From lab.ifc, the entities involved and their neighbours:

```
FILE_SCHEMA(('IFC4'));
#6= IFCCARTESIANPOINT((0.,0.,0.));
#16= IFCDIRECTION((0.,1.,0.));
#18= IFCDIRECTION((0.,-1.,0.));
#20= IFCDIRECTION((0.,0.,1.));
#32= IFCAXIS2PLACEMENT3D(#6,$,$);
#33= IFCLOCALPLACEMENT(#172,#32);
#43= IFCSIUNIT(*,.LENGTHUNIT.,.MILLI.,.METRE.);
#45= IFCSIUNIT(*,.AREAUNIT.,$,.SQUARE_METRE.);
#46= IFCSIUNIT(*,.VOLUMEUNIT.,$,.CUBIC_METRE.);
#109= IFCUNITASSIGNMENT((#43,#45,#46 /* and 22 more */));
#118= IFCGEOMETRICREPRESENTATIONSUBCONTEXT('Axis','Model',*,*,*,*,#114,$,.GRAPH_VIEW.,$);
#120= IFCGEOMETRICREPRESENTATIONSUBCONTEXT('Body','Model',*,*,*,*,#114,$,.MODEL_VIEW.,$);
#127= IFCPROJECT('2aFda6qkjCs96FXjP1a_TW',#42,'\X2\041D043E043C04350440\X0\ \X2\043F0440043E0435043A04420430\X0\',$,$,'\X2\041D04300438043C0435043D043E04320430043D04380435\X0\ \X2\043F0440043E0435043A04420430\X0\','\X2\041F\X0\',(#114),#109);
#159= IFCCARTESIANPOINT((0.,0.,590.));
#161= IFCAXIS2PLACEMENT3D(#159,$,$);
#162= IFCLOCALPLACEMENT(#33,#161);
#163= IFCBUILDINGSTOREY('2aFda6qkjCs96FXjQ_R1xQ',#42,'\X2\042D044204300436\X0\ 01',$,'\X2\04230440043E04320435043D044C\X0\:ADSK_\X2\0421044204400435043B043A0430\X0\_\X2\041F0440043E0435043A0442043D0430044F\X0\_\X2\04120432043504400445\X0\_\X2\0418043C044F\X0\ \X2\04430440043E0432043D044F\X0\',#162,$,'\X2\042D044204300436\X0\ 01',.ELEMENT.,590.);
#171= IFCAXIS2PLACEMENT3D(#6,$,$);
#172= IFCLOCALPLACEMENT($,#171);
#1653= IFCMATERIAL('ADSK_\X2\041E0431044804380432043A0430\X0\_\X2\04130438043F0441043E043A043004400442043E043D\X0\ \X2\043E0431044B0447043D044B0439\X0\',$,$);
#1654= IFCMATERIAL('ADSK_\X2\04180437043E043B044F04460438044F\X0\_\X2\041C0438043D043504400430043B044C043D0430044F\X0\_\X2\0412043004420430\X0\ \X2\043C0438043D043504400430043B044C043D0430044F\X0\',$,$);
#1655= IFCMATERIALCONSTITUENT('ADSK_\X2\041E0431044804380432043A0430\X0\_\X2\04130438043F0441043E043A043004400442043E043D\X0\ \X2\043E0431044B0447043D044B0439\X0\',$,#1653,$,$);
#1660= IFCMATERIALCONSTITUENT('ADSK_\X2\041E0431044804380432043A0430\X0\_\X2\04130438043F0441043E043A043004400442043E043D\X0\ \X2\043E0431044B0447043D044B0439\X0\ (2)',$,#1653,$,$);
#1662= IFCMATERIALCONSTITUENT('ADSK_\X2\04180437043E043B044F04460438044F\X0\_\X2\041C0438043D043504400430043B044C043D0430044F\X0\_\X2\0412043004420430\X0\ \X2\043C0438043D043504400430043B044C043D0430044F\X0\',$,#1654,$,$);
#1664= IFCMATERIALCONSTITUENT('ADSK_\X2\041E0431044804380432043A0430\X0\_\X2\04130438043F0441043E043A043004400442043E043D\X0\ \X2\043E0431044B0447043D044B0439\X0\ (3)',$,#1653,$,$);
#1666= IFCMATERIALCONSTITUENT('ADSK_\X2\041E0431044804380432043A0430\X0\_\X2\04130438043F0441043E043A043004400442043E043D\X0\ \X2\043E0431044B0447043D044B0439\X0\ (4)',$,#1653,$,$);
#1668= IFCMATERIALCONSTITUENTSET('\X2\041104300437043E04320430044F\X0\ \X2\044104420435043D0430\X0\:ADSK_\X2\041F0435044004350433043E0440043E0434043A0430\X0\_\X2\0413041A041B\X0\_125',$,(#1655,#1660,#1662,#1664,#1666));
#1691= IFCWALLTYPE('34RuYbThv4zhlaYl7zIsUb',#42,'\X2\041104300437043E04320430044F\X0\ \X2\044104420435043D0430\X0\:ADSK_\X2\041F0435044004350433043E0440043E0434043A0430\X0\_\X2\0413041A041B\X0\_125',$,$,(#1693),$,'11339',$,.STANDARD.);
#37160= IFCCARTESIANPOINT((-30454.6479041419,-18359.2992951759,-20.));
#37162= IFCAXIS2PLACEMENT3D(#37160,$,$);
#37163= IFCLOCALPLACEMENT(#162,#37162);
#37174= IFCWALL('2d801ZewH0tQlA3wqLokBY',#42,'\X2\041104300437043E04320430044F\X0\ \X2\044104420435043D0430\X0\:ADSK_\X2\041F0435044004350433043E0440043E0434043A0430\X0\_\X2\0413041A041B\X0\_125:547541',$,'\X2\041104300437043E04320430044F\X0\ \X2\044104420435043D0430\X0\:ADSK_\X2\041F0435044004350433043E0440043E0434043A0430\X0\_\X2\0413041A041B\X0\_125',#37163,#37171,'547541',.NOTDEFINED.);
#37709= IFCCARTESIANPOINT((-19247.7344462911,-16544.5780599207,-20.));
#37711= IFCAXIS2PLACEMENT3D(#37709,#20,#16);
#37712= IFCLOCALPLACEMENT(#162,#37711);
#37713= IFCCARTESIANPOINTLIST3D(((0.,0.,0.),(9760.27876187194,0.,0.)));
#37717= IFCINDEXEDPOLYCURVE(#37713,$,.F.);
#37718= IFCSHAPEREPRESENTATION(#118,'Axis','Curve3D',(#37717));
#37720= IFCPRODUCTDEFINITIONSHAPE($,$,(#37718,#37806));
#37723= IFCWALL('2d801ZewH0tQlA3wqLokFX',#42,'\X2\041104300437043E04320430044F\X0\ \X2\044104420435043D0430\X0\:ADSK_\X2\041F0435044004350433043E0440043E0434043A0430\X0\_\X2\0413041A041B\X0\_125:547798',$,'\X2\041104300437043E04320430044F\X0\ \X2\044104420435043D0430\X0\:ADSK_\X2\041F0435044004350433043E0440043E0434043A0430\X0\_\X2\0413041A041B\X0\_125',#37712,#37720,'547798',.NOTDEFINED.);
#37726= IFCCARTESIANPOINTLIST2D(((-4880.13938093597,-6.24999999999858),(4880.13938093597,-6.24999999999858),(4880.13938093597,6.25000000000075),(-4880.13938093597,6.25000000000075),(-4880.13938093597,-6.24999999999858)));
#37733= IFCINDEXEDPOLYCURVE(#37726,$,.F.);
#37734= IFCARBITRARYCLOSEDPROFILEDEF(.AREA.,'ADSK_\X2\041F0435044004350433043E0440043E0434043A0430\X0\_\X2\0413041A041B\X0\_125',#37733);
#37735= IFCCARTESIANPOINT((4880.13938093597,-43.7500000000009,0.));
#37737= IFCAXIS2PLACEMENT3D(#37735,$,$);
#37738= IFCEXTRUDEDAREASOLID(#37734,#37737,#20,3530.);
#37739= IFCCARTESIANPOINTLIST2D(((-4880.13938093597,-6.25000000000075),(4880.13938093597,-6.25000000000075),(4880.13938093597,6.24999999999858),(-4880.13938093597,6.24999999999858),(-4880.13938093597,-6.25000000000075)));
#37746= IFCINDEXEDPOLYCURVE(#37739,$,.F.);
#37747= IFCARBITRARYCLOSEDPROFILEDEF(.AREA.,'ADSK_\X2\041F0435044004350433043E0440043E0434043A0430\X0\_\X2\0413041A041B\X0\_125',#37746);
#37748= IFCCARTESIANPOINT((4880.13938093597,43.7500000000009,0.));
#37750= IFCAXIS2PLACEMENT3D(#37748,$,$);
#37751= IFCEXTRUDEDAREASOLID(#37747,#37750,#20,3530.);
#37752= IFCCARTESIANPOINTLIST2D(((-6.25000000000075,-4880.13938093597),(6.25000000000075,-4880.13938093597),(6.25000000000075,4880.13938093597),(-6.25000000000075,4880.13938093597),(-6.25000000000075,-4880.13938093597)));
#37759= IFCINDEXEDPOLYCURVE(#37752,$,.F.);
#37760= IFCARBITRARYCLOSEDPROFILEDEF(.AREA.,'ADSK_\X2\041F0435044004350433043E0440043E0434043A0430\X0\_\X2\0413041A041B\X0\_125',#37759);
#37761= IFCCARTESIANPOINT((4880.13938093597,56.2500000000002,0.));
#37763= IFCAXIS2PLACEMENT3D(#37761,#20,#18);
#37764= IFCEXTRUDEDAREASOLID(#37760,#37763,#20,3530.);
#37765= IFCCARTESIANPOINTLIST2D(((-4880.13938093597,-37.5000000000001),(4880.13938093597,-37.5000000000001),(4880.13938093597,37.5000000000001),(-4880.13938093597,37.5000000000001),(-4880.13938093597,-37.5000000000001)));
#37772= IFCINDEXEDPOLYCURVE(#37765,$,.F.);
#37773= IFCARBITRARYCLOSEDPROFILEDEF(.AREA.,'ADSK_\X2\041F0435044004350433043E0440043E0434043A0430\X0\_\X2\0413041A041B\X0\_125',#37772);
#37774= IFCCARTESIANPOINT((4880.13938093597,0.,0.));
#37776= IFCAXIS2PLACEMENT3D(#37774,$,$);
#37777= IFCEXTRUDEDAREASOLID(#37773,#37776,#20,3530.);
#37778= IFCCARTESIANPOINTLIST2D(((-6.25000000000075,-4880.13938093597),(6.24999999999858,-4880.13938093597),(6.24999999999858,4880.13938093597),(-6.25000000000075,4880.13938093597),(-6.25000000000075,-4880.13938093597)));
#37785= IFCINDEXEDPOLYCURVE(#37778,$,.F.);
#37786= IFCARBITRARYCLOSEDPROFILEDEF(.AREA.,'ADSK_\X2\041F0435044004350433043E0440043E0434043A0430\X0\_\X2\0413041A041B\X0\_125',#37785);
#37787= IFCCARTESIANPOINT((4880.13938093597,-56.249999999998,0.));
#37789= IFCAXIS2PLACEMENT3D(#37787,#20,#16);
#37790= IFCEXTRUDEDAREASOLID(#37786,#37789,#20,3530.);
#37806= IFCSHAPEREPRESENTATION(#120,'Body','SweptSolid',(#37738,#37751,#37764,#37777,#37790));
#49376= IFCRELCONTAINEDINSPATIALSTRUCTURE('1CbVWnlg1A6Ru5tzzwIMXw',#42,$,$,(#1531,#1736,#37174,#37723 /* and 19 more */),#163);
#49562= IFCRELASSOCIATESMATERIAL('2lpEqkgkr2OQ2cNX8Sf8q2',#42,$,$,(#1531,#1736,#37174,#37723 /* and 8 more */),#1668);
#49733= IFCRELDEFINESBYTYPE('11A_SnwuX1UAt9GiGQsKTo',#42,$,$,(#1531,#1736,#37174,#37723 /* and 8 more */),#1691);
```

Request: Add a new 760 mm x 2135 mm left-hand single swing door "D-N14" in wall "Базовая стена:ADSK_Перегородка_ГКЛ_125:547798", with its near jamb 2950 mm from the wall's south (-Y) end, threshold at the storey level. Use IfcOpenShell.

```python
import numpy as np
import ifcopenshell
import ifcopenshell.api.feature
import ifcopenshell.api.geometry
import ifcopenshell.api.root
import ifcopenshell.api.spatial
import ifcopenshell.geom
import ifcopenshell.util.element
import ifcopenshell.util.placement
import ifcopenshell.util.representation
import ifcopenshell.util.shape
import ifcopenshell.util.unit

model = ifcopenshell.open("lab.ifc")
unit_scale = ifcopenshell.util.unit.calculate_unit_scale(model)
settings = ifcopenshell.geom.settings()


def volume(element):
    """Net volume in cubic metres, openings subtracted."""
    shape = ifcopenshell.geom.create_shape(settings, element)
    return ifcopenshell.util.shape.get_volume(shape.geometry)


wall = model.by_guid("2d801ZewH0tQlA3wqLokFX")
storey = ifcopenshell.util.element.get_container(wall, ifc_class="IfcBuildingStorey")
context = ifcopenshell.util.representation.get_context(model, "Model", "Body", "MODEL_VIEW")
before = volume(wall)

width, height, from_end, sill = 0.76, 2.135, 2.95, 0.0  # metres

# The wall runs along its own X axis, and the end named is its -X end.
wall_shape = ifcopenshell.geom.create_shape(settings, wall)
x, y, z = ifcopenshell.util.shape.get_vertices(wall_shape.geometry).T
start = x.min() + from_end
face, thickness = float(y.min()), float(y.max() - y.min())
wall_matrix = ifcopenshell.util.placement.get_local_placement(wall.ObjectPlacement)
level = ifcopenshell.util.placement.get_local_placement(storey.ObjectPlacement)[2, 3]


def in_wall(x, y):
    """Placement at x, y metres in the wall's axes, at sill height."""
    matrix = wall_matrix.copy()
    matrix[:, 3] = wall_matrix @ np.array([x / unit_scale, y / unit_scale, 0.0, 1.0])
    matrix[2, 3] = level + sill / unit_scale
    return matrix


# Opening: a box that overshoots both wall faces by 50 mm.
opening = ifcopenshell.api.root.create_entity(model, ifc_class="IfcOpeningElement", predefined_type="OPENING")
box = ifcopenshell.api.geometry.add_wall_representation(
    model, context=context, length=width, height=height, thickness=thickness + 0.1
)
ifcopenshell.api.geometry.assign_representation(model, product=opening, representation=box)
ifcopenshell.api.geometry.edit_object_placement(model, product=opening, matrix=in_wall(start, face - 0.05), is_si=False)
ifcopenshell.api.feature.add_feature(model, feature=opening, element=wall)

door = ifcopenshell.api.root.create_entity(model, ifc_class="IfcDoor", name="D-N14", predefined_type="DOOR")
door.OverallWidth, door.OverallHeight = width / unit_scale, height / unit_scale
door.OperationType = "SINGLE_SWING_LEFT"
body = ifcopenshell.api.geometry.add_door_representation(
    model,
    context=context,
    overall_width=door.OverallWidth,
    overall_height=door.OverallHeight,
    operation_type="SINGLE_SWING_LEFT",
    lining_properties={"LiningDepth": thickness / unit_scale, "ThresholdDepth": thickness / unit_scale},
)
ifcopenshell.api.geometry.assign_representation(model, product=door, representation=body)
ifcopenshell.api.spatial.assign_container(model, products=[door], relating_structure=storey)
ifcopenshell.api.feature.add_filling(model, opening=opening, element=door)

# The lining spans the wall, so the door starts at the wall face.
ifcopenshell.api.geometry.edit_object_placement(model, product=door, matrix=in_wall(start, face), is_si=False)

after = volume(wall)

print(f"wall volume {before:.3f} -> {after:.3f} m3")

model.write("lab_updated.ifc")
```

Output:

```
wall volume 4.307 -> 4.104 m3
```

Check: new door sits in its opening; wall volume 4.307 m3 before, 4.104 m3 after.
